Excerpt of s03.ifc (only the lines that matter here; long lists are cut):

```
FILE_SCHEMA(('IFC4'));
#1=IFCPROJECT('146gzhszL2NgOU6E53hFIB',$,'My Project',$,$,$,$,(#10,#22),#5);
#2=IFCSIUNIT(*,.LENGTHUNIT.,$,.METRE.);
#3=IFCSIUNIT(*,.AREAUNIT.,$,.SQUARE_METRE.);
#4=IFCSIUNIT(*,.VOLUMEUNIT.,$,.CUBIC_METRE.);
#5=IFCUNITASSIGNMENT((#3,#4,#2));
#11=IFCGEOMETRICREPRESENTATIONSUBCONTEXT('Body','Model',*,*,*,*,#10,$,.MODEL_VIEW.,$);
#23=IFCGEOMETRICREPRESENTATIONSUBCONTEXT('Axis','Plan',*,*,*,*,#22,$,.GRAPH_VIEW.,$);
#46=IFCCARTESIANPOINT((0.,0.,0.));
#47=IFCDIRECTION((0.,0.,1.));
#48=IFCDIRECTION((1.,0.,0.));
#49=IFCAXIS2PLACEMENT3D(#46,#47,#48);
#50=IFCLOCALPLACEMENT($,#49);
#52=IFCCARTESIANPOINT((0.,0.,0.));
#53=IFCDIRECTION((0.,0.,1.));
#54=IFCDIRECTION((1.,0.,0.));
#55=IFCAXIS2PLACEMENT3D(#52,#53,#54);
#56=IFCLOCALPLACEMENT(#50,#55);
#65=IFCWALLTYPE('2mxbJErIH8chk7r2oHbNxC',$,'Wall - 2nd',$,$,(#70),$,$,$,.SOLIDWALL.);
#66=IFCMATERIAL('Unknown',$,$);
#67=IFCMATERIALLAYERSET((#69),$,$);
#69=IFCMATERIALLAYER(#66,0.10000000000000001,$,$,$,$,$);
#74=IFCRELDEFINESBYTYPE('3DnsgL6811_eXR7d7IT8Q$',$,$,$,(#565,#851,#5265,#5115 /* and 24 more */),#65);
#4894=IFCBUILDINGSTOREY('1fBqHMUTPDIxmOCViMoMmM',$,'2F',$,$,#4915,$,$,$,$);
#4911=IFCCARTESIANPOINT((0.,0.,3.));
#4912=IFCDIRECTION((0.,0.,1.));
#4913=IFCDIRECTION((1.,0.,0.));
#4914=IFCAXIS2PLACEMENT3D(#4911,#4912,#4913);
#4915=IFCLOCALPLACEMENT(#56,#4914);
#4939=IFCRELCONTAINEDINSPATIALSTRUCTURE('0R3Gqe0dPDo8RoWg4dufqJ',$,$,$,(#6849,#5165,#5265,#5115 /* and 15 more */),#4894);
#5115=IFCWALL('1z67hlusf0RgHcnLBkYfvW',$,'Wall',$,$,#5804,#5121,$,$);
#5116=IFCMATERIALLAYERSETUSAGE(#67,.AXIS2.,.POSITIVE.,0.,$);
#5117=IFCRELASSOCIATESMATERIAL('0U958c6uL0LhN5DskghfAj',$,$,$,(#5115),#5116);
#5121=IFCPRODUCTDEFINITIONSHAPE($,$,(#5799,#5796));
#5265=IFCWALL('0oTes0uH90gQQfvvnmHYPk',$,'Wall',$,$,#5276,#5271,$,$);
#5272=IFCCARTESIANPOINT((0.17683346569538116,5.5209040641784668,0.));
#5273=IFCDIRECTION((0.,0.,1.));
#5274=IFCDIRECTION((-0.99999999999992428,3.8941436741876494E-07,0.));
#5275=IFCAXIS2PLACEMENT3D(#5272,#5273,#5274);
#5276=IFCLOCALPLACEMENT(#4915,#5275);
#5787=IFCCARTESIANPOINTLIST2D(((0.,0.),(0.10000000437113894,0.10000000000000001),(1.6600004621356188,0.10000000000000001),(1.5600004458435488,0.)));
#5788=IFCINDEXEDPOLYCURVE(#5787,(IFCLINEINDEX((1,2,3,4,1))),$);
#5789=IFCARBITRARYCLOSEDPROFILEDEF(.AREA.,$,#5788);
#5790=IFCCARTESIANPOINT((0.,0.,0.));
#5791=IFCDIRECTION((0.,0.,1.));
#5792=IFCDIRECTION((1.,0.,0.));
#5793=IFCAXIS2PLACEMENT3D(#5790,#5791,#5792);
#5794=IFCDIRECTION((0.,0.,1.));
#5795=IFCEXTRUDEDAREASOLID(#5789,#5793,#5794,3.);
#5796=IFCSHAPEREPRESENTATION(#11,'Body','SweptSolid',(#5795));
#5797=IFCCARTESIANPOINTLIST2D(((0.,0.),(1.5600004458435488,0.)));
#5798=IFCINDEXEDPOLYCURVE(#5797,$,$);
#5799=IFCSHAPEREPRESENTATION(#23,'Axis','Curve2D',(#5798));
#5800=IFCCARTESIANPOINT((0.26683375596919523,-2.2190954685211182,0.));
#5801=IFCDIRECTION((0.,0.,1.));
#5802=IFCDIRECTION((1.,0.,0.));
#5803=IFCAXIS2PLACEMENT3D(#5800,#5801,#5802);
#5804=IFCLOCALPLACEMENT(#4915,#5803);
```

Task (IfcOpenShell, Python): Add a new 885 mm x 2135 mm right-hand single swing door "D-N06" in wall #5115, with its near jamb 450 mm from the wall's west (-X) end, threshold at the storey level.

```python
import numpy as np
import ifcopenshell
import ifcopenshell.api.feature
import ifcopenshell.api.geometry
import ifcopenshell.api.root
import ifcopenshell.api.spatial
import ifcopenshell.geom
import ifcopenshell.util.element
import ifcopenshell.util.placement
import ifcopenshell.util.representation
import ifcopenshell.util.shape
import ifcopenshell.util.unit

model = ifcopenshell.open("s03.ifc")
unit_scale = ifcopenshell.util.unit.calculate_unit_scale(model)
settings = ifcopenshell.geom.settings()


def volume(element):
    """Net volume in cubic metres, openings subtracted."""
    shape = ifcopenshell.geom.create_shape(settings, element)
    return ifcopenshell.util.shape.get_volume(shape.geometry)


wall = model.by_guid("1z67hlusf0RgHcnLBkYfvW")
storey = ifcopenshell.util.element.get_container(wall, ifc_class="IfcBuildingStorey")
context = ifcopenshell.util.representation.get_context(model, "Model", "Body", "MODEL_VIEW")
before = volume(wall)

width, height, from_end, sill = 0.885, 2.135, 0.45, 0.0  # metres

# The wall runs along its own X axis, and the end named is its -X end.
wall_shape = ifcopenshell.geom.create_shape(settings, wall)
x, y, z = ifcopenshell.util.shape.get_vertices(wall_shape.geometry).T
start = x.min() + from_end
face, thickness = float(y.min()), float(y.max() - y.min())
wall_matrix = ifcopenshell.util.placement.get_local_placement(wall.ObjectPlacement)
level = ifcopenshell.util.placement.get_local_placement(storey.ObjectPlacement)[2, 3]


def in_wall(x, y):
    """Placement at x, y metres in the wall's axes, at sill height."""
    matrix = wall_matrix.copy()
    matrix[:, 3] = wall_matrix @ np.array([x / unit_scale, y / unit_scale, 0.0, 1.0])
    matrix[2, 3] = level + sill / unit_scale
    return matrix


# Opening: a box that overshoots both wall faces by 50 mm.
opening = ifcopenshell.api.root.create_entity(model, ifc_class="IfcOpeningElement", predefined_type="OPENING")
box = ifcopenshell.api.geometry.add_wall_representation(
    model, context=context, length=width, height=height, thickness=thickness + 0.1
)
ifcopenshell.api.geometry.assign_representation(model, product=opening, representation=box)
ifcopenshell.api.geometry.edit_object_placement(model, product=opening, matrix=in_wall(start, face - 0.05), is_si=False)
ifcopenshell.api.feature.add_feature(model, feature=opening, element=wall)

door = ifcopenshell.api.root.create_entity(model, ifc_class="IfcDoor", name="D-N06", predefined_type="DOOR")
door.OverallWidth, door.OverallHeight = width / unit_scale, height / unit_scale
door.OperationType = "SINGLE_SWING_RIGHT"
body = ifcopenshell.api.geometry.add_door_representation(
    model,
    context=context,
    overall_width=door.OverallWidth,
    overall_height=door.OverallHeight,
    operation_type="SINGLE_SWING_RIGHT",
    lining_properties={"LiningDepth": thickness / unit_scale, "ThresholdDepth": thickness / unit_scale},
)
ifcopenshell.api.geometry.assign_representation(model, product=door, representation=body)
ifcopenshell.api.spatial.assign_container(model, products=[door], relating_structure=storey)
ifcopenshell.api.feature.add_filling(model, opening=opening, element=door)

# The lining spans the wall, so the door starts at the wall face.
ifcopenshell.api.geometry.edit_object_placement(model, product=door, matrix=in_wall(start, face), is_si=False)

after = volume(wall)

print(f"wall volume {before:.3f} -> {after:.3f} m3")

model.write("s03_v2.ifc")
```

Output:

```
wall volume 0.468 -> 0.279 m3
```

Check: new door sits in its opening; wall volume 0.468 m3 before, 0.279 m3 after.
